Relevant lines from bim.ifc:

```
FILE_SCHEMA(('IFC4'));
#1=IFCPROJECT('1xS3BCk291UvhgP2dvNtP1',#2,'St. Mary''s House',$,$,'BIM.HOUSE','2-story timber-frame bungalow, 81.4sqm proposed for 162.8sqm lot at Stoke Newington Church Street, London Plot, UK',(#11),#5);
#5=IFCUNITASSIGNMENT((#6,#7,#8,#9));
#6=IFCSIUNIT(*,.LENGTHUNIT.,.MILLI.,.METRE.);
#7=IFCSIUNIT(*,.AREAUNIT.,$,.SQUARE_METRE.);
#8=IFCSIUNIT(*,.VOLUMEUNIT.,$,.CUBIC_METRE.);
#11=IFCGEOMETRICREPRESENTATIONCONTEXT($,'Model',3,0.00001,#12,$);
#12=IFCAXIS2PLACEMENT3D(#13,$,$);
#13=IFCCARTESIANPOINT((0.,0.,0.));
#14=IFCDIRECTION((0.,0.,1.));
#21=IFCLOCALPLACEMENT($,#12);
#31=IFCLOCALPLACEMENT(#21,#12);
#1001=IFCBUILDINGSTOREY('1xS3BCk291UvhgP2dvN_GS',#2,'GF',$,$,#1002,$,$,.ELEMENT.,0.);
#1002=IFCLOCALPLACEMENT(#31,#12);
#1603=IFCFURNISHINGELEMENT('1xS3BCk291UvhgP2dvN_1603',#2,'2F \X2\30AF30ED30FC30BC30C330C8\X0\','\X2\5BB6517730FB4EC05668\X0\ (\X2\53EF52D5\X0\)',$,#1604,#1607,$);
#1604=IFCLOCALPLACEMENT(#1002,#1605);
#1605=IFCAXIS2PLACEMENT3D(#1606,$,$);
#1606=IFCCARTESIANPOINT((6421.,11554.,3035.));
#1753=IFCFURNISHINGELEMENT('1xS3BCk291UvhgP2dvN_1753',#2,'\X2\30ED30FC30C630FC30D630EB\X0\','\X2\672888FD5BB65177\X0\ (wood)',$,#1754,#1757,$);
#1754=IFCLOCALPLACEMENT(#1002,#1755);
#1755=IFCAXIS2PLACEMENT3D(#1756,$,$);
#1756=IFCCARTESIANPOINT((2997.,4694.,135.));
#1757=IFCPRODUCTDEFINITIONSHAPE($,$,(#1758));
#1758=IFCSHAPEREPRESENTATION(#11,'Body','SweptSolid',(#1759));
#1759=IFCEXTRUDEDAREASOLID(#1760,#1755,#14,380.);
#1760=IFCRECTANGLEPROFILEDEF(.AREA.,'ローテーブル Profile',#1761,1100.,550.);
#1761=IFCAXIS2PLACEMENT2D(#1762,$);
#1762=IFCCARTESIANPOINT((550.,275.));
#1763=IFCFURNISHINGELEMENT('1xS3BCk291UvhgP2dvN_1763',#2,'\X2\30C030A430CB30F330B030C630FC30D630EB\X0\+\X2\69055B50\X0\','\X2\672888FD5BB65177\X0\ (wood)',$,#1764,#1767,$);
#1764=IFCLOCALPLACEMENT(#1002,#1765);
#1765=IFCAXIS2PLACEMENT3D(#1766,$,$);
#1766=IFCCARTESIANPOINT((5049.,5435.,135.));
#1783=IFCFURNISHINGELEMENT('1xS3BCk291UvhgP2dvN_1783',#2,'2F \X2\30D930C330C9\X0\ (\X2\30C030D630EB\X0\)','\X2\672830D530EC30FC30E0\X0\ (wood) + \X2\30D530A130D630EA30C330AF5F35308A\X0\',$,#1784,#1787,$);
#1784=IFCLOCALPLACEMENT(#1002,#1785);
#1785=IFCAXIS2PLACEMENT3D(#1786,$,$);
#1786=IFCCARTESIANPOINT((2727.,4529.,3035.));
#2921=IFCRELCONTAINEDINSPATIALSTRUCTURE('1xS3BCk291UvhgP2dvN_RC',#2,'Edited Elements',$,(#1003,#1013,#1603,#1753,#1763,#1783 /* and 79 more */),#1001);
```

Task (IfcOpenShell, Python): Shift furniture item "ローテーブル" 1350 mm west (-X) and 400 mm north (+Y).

```python
import ifcopenshell
import ifcopenshell.api.geometry
import ifcopenshell.util.placement
import ifcopenshell.util.unit

model = ifcopenshell.open("bim.ifc")
unit_scale = ifcopenshell.util.unit.calculate_unit_scale(model)

item = model.by_guid("1xS3BCk291UvhgP2dvN_1753")
matrix = ifcopenshell.util.placement.get_local_placement(item.ObjectPlacement)
matrix[0, 3] -= 1.35 / unit_scale
matrix[1, 3] += 0.4 / unit_scale
ifcopenshell.api.geometry.edit_object_placement(model, product=item, matrix=matrix, is_si=False)

print(ifcopenshell.util.placement.get_local_placement(item.ObjectPlacement).round(3) + 0.0)

model.write("bim_edited.ifc")
```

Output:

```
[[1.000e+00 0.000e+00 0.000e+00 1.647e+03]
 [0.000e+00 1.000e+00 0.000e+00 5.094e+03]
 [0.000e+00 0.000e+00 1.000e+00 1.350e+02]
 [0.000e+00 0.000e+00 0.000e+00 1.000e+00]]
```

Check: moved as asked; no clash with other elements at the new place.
